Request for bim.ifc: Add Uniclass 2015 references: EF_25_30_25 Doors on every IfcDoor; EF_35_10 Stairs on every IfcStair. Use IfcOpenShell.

First a look at what the model holds.

```python
import ifcopenshell

model = ifcopenshell.open("bim.ifc")
print(model.schema)
print("classifications:", [c.Name for c in model.by_type("IfcClassification")])
for ifc_class in ("IfcDoor", "IfcRoof", "IfcStair", "IfcWall", "IfcWindow"):
    print(ifc_class, len(model.by_type(ifc_class)))
```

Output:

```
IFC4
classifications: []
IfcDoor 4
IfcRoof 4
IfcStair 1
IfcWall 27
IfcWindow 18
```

```python
import ifcopenshell
import ifcopenshell.api.classification

model = ifcopenshell.open("bim.ifc")

system = ifcopenshell.api.classification.add_classification(model, classification="Uniclass 2015")

codes = {
    "IfcDoor": ("EF_25_30_25", "Doors"),
    "IfcStair": ("EF_35_10", "Stairs"),
}
for ifc_class, (code, name) in codes.items():
    products = model.by_type(ifc_class)
    ifcopenshell.api.classification.add_reference(
        model, products=products, classification=system, identification=code, name=name
    )
    print(code, len(products))

model.write("bim_edited.ifc")
```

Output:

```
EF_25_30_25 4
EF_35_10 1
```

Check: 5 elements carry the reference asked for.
